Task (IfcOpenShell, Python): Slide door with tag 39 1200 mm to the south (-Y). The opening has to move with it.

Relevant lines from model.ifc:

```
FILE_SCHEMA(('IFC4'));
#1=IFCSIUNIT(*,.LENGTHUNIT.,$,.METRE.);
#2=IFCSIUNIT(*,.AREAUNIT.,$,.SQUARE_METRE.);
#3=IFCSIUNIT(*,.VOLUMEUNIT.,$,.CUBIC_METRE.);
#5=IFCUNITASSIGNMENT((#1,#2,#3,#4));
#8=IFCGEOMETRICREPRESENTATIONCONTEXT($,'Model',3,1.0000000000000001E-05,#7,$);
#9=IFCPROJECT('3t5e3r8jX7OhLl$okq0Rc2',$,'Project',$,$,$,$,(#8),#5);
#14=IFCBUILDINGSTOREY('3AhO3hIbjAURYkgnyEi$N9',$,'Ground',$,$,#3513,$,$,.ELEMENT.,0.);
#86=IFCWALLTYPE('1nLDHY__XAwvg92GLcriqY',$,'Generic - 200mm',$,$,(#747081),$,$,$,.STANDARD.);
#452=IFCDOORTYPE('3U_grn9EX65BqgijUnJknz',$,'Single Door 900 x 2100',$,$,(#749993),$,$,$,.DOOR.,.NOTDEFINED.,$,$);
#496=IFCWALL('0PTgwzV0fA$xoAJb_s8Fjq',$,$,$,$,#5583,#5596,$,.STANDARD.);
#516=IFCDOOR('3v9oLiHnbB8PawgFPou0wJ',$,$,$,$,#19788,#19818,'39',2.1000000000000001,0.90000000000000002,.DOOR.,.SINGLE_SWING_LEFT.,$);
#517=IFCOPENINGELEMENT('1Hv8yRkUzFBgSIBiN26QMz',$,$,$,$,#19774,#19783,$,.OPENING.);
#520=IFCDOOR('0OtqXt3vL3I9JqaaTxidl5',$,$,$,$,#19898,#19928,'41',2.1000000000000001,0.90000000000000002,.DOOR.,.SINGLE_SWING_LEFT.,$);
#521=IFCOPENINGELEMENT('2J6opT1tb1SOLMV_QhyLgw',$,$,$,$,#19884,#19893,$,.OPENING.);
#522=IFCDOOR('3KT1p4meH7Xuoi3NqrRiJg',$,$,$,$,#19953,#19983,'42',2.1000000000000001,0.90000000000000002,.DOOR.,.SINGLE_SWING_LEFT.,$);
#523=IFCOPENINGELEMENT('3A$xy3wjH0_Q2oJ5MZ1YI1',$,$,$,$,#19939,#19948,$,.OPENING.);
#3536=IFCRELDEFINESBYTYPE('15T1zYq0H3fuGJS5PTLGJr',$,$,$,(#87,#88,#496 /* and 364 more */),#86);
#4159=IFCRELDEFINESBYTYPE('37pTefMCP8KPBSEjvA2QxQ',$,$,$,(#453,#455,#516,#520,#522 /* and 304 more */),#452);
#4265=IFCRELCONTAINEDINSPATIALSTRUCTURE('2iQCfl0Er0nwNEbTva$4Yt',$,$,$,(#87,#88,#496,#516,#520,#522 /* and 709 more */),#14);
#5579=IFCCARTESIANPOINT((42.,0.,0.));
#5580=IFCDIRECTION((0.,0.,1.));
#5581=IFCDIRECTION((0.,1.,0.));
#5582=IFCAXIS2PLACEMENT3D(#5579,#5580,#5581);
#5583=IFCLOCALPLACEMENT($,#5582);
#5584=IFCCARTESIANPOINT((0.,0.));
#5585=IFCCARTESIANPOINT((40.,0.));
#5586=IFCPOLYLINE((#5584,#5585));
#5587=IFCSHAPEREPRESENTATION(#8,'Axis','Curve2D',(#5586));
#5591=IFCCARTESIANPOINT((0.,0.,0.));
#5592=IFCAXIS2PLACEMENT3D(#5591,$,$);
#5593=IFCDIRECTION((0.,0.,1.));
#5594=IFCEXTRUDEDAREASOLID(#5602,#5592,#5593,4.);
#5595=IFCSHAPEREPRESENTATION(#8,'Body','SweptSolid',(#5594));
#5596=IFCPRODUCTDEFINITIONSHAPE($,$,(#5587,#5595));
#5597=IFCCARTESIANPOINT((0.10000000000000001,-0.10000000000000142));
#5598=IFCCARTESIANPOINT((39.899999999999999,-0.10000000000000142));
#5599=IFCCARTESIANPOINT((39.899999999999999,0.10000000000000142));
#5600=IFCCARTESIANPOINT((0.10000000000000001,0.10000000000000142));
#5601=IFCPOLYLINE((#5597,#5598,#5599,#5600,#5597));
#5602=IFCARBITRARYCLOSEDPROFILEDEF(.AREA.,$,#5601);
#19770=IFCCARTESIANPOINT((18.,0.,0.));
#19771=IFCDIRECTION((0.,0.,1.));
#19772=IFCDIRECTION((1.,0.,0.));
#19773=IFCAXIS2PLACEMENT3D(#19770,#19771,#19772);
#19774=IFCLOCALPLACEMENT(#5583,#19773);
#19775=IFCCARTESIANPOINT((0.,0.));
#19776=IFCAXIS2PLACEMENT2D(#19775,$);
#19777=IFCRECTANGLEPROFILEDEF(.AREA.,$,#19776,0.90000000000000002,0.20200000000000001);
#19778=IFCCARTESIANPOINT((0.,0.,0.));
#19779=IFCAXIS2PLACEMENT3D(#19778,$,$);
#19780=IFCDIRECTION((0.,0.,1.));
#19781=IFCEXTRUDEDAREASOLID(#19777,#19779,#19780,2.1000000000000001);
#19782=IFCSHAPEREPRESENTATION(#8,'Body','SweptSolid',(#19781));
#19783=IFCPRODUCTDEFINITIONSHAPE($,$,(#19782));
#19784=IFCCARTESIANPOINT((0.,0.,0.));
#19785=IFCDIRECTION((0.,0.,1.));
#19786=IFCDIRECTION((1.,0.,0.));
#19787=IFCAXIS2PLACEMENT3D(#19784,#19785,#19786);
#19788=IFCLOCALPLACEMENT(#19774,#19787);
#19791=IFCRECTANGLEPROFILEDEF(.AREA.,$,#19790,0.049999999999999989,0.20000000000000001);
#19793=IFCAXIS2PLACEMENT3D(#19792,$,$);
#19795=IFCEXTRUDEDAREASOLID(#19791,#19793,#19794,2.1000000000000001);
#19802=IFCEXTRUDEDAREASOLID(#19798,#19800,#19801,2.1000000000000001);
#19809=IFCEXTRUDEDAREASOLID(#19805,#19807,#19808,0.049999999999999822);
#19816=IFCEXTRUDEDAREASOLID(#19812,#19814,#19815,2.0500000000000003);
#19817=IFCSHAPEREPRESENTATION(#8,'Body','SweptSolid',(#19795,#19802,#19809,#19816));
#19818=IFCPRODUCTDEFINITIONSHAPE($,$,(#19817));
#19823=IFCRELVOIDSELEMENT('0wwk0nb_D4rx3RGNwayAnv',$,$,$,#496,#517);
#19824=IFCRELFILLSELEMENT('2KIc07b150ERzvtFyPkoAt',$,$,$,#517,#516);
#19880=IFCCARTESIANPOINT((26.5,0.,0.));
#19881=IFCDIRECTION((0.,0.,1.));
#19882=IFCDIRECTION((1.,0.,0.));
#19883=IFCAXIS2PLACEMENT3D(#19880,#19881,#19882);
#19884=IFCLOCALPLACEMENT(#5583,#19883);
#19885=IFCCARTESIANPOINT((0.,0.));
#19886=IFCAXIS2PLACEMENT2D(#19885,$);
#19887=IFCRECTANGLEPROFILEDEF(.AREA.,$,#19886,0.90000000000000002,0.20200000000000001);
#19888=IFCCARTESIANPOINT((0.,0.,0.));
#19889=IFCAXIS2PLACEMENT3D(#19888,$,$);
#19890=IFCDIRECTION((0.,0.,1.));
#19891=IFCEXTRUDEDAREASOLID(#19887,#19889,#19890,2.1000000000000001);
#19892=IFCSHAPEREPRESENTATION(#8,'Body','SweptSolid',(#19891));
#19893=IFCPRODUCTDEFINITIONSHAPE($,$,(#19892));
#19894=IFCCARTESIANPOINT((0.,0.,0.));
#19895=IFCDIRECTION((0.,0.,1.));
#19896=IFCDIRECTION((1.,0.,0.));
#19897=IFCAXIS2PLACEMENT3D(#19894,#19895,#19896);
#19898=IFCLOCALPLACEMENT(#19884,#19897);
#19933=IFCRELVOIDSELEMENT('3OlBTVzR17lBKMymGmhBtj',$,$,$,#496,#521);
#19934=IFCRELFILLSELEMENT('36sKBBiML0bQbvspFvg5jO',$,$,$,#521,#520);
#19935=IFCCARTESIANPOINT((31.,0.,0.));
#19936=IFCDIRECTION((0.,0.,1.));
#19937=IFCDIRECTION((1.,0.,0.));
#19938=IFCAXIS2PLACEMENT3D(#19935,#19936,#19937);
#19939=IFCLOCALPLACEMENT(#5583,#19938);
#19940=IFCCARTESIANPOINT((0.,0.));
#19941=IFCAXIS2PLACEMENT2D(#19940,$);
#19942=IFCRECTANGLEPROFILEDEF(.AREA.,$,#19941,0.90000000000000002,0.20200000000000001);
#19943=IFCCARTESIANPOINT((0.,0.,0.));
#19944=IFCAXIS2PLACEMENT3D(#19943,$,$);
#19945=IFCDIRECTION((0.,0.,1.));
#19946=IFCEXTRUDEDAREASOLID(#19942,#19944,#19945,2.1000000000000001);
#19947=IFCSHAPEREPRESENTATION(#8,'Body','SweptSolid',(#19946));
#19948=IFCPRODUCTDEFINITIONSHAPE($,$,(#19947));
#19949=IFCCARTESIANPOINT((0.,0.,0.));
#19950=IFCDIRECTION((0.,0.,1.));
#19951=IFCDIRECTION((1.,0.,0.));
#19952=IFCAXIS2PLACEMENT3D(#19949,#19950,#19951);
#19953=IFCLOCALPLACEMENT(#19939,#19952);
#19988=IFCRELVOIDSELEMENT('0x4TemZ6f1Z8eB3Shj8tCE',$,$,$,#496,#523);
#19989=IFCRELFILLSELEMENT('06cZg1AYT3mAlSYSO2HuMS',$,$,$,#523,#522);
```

```python
import ifcopenshell
import ifcopenshell.api.geometry
import ifcopenshell.util.placement
import ifcopenshell.util.unit

model = ifcopenshell.open("model.ifc")
unit_scale = ifcopenshell.util.unit.calculate_unit_scale(model)

door = model.by_guid("3v9oLiHnbB8PawgFPou0wJ")
opening = door.FillsVoids[0].RelatingOpeningElement
wall = opening.VoidsElements[0].RelatingBuildingElement

wall_matrix = ifcopenshell.util.placement.get_local_placement(wall.ObjectPlacement)
shift = wall_matrix[:3, 0] * -1.2 / unit_scale
before = ifcopenshell.util.placement.get_local_placement(door.ObjectPlacement)[:3, 3].copy()

# The door is placed relative to its opening, so it follows when the opening moves.
matrix = ifcopenshell.util.placement.get_local_placement(opening.ObjectPlacement)
matrix[:3, 3] += shift
ifcopenshell.api.geometry.edit_object_placement(
    model, product=opening, matrix=matrix, is_si=False, should_transform_children=True
)

after = ifcopenshell.util.placement.get_local_placement(door.ObjectPlacement)[:3, 3]
print("door moved by", (after - before).round(3) + 0.0)

model.write("model_v2.ifc")
```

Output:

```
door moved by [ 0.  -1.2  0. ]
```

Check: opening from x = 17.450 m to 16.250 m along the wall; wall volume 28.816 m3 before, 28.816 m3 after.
